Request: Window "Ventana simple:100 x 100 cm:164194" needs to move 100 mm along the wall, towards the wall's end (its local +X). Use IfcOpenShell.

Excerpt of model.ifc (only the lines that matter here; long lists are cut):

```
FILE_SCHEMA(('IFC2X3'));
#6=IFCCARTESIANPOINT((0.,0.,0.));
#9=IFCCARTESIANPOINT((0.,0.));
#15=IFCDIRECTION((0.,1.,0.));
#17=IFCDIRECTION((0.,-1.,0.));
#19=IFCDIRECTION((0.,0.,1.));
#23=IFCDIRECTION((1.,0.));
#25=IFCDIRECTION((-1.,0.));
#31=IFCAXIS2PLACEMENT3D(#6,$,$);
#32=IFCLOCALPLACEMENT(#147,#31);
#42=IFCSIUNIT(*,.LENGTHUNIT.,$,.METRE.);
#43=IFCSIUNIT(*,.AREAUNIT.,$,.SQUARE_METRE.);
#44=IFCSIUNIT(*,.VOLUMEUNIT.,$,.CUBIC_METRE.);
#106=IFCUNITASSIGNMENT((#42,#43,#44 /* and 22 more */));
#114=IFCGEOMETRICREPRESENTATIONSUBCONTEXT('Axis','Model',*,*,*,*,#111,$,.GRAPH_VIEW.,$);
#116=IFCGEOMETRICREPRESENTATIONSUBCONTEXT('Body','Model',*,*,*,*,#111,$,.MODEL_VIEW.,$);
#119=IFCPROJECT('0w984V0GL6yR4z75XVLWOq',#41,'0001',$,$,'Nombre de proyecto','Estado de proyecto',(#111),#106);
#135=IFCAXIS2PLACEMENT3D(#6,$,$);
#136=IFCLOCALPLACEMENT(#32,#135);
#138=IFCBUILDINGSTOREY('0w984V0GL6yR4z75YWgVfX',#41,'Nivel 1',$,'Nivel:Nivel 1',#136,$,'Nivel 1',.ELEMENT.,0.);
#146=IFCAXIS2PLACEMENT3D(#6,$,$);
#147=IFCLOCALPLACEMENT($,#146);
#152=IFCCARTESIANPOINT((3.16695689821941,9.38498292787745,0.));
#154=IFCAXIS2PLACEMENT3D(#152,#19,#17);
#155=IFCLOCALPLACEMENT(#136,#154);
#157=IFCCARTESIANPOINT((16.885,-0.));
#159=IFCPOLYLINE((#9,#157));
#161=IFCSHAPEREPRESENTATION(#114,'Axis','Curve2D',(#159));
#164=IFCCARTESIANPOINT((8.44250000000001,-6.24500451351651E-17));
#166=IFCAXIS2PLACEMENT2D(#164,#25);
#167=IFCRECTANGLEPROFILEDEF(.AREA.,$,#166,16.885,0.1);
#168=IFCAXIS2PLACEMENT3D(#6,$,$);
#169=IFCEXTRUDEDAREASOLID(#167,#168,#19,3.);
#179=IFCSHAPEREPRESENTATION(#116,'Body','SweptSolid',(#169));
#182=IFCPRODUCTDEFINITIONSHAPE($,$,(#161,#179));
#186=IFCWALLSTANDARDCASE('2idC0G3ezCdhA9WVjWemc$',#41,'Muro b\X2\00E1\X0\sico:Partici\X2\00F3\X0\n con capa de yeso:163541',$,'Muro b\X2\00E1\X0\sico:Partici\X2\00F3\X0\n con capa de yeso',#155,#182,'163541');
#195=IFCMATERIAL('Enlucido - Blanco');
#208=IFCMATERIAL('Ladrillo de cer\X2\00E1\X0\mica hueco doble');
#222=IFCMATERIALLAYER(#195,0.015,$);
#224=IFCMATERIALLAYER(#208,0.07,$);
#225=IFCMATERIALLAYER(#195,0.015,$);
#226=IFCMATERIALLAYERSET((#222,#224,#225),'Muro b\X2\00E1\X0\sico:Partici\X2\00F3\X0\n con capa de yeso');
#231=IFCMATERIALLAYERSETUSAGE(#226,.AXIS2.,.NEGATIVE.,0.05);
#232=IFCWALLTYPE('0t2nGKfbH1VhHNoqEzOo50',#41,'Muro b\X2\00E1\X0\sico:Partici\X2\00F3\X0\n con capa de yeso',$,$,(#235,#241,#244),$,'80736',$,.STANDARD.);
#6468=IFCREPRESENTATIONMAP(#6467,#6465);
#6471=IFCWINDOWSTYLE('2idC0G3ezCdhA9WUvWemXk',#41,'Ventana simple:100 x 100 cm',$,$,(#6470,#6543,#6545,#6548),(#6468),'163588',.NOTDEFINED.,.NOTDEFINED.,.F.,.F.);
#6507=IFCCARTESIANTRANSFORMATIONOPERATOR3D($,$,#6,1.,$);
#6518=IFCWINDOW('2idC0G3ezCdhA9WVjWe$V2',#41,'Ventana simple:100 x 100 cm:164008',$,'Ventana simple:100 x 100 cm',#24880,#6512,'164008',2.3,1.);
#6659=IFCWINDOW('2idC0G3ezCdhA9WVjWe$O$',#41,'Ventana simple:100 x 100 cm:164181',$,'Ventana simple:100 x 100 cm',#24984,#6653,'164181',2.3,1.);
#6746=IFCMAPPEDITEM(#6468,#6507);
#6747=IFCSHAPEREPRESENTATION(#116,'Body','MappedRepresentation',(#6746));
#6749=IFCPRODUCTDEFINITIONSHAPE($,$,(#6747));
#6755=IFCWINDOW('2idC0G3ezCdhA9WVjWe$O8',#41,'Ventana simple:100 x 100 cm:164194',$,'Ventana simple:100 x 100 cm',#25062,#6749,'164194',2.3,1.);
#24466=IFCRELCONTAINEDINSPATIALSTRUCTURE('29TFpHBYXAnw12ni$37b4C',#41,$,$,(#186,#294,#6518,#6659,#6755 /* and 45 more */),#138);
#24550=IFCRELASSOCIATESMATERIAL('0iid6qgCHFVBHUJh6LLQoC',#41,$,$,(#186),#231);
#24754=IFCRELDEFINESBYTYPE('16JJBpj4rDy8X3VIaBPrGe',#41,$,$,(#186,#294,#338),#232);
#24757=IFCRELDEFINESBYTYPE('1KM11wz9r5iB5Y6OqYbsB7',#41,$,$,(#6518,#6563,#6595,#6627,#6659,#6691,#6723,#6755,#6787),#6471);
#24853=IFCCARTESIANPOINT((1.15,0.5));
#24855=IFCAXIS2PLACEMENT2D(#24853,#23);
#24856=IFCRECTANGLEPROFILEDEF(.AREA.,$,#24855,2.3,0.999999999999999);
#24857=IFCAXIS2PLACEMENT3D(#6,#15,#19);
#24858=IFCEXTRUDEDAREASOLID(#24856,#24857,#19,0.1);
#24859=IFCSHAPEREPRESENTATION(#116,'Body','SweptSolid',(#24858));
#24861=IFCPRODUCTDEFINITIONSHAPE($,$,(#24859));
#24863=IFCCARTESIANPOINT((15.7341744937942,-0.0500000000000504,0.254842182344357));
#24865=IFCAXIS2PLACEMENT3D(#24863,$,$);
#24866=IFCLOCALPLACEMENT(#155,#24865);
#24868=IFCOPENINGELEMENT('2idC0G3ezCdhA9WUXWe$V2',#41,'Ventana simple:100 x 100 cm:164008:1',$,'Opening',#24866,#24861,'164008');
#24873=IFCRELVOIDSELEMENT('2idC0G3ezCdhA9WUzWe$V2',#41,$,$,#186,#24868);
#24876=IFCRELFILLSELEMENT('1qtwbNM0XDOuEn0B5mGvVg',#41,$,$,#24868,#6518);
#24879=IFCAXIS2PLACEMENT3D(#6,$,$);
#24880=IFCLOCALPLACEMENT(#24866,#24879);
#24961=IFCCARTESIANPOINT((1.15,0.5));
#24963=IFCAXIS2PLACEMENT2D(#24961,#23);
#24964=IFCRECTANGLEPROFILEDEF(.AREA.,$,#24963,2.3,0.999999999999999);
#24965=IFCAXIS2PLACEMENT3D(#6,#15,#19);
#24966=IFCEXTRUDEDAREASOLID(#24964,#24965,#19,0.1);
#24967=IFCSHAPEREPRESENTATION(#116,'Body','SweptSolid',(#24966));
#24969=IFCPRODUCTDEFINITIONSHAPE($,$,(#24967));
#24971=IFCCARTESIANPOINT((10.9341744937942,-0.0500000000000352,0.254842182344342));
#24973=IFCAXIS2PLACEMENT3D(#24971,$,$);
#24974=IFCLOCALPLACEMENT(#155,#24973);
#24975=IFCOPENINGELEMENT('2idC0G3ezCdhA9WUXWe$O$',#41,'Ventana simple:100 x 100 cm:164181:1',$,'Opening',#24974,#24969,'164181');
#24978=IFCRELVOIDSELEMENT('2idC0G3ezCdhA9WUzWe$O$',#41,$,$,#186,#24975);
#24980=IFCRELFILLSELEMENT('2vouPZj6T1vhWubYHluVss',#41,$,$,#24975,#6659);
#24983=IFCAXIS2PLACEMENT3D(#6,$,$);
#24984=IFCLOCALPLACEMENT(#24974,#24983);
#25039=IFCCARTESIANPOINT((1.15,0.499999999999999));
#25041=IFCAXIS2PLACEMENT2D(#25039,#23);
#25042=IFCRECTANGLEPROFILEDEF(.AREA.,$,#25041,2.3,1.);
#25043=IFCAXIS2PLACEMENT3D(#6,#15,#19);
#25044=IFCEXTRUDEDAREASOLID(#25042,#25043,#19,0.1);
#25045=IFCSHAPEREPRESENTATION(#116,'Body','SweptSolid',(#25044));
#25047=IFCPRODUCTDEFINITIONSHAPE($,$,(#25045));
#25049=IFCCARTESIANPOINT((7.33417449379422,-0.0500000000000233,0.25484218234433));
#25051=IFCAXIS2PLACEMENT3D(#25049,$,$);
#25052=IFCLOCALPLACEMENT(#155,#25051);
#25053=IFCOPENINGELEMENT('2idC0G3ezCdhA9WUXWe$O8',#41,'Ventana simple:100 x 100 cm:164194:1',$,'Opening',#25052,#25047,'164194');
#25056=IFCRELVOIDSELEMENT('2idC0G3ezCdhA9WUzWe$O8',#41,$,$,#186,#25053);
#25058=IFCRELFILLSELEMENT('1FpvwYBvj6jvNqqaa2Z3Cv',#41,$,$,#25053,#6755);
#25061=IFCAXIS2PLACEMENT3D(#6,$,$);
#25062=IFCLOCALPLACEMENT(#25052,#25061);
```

```python
import ifcopenshell
import ifcopenshell.api.geometry
import ifcopenshell.util.placement
import ifcopenshell.util.unit

model = ifcopenshell.open("model.ifc")
unit_scale = ifcopenshell.util.unit.calculate_unit_scale(model)

window = model.by_guid("2idC0G3ezCdhA9WVjWe$O8")
opening = window.FillsVoids[0].RelatingOpeningElement
wall = opening.VoidsElements[0].RelatingBuildingElement

wall_matrix = ifcopenshell.util.placement.get_local_placement(wall.ObjectPlacement)
shift = wall_matrix[:3, 0] * 0.1 / unit_scale
before = ifcopenshell.util.placement.get_local_placement(window.ObjectPlacement)[:3, 3].copy()

# The window is placed relative to its opening, so it follows when the opening moves.
matrix = ifcopenshell.util.placement.get_local_placement(opening.ObjectPlacement)
matrix[:3, 3] += shift
ifcopenshell.api.geometry.edit_object_placement(
    model, product=opening, matrix=matrix, is_si=False, should_transform_children=True
)

after = ifcopenshell.util.placement.get_local_placement(window.ObjectPlacement)[:3, 3]
print("window moved by", (after - before).round(3) + 0.0)

model.write("model_v2.ifc")
```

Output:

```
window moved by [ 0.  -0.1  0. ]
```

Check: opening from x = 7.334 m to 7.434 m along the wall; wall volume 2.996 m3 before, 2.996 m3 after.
